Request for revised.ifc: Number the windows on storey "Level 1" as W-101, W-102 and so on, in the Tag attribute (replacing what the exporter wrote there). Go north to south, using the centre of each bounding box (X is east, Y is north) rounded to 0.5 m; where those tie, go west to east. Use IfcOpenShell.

First a look at what the model holds.

```python
import ifcopenshell
import ifcopenshell.util.element
import ifcopenshell.util.placement

model = ifcopenshell.open("revised.ifc")
print(model.schema)
storey = next(s for s in model.by_type("IfcBuildingStorey") if s.Name == "Level 1")
windows = [e for e in ifcopenshell.util.element.get_decomposition(storey) if e.is_a("IfcWindow")]
for e in sorted(windows, key=lambda e: e.id()):
    origin = ifcopenshell.util.placement.get_local_placement(e.ObjectPlacement)[:3, 3]
    print(e.id(), e.Tag, e.Name, origin.round(2) + 0.0, sep=" | ")
```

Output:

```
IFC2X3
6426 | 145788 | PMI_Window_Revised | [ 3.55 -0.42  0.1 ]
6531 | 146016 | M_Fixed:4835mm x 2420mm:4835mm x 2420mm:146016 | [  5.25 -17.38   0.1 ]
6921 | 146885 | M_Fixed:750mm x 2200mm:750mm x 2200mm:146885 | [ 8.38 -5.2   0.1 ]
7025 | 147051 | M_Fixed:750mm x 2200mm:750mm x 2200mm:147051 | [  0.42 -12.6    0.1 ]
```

```python
import ifcopenshell
import ifcopenshell.geom
import ifcopenshell.util.element
import ifcopenshell.util.shape

model = ifcopenshell.open("revised.ifc")
settings = ifcopenshell.geom.settings()
settings.set("use-world-coords", True)


def centre(element):
    shape = ifcopenshell.geom.create_shape(settings, element)
    return ifcopenshell.util.shape.get_bbox_centroid(shape.geometry)


storey = next(s for s in model.by_type("IfcBuildingStorey") if s.Name == "Level 1")
windows = [e for e in ifcopenshell.util.element.get_decomposition(storey) if e.is_a("IfcWindow")]

# Insertion points can sit at a corner or the storey origin, so sort by the geometry (in metres).
centres = {e: centre(e) for e in windows}
windows.sort(key=lambda e: (-round(centres[e][1] / 0.5), centres[e][0]))

for i, e in enumerate(windows, start=1):
    number = f"W-1{i:02d}"
    e.Tag = number
    print(e.id(), number)

model.write("revised_v2.ifc")
```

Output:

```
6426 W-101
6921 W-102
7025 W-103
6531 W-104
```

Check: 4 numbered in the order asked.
